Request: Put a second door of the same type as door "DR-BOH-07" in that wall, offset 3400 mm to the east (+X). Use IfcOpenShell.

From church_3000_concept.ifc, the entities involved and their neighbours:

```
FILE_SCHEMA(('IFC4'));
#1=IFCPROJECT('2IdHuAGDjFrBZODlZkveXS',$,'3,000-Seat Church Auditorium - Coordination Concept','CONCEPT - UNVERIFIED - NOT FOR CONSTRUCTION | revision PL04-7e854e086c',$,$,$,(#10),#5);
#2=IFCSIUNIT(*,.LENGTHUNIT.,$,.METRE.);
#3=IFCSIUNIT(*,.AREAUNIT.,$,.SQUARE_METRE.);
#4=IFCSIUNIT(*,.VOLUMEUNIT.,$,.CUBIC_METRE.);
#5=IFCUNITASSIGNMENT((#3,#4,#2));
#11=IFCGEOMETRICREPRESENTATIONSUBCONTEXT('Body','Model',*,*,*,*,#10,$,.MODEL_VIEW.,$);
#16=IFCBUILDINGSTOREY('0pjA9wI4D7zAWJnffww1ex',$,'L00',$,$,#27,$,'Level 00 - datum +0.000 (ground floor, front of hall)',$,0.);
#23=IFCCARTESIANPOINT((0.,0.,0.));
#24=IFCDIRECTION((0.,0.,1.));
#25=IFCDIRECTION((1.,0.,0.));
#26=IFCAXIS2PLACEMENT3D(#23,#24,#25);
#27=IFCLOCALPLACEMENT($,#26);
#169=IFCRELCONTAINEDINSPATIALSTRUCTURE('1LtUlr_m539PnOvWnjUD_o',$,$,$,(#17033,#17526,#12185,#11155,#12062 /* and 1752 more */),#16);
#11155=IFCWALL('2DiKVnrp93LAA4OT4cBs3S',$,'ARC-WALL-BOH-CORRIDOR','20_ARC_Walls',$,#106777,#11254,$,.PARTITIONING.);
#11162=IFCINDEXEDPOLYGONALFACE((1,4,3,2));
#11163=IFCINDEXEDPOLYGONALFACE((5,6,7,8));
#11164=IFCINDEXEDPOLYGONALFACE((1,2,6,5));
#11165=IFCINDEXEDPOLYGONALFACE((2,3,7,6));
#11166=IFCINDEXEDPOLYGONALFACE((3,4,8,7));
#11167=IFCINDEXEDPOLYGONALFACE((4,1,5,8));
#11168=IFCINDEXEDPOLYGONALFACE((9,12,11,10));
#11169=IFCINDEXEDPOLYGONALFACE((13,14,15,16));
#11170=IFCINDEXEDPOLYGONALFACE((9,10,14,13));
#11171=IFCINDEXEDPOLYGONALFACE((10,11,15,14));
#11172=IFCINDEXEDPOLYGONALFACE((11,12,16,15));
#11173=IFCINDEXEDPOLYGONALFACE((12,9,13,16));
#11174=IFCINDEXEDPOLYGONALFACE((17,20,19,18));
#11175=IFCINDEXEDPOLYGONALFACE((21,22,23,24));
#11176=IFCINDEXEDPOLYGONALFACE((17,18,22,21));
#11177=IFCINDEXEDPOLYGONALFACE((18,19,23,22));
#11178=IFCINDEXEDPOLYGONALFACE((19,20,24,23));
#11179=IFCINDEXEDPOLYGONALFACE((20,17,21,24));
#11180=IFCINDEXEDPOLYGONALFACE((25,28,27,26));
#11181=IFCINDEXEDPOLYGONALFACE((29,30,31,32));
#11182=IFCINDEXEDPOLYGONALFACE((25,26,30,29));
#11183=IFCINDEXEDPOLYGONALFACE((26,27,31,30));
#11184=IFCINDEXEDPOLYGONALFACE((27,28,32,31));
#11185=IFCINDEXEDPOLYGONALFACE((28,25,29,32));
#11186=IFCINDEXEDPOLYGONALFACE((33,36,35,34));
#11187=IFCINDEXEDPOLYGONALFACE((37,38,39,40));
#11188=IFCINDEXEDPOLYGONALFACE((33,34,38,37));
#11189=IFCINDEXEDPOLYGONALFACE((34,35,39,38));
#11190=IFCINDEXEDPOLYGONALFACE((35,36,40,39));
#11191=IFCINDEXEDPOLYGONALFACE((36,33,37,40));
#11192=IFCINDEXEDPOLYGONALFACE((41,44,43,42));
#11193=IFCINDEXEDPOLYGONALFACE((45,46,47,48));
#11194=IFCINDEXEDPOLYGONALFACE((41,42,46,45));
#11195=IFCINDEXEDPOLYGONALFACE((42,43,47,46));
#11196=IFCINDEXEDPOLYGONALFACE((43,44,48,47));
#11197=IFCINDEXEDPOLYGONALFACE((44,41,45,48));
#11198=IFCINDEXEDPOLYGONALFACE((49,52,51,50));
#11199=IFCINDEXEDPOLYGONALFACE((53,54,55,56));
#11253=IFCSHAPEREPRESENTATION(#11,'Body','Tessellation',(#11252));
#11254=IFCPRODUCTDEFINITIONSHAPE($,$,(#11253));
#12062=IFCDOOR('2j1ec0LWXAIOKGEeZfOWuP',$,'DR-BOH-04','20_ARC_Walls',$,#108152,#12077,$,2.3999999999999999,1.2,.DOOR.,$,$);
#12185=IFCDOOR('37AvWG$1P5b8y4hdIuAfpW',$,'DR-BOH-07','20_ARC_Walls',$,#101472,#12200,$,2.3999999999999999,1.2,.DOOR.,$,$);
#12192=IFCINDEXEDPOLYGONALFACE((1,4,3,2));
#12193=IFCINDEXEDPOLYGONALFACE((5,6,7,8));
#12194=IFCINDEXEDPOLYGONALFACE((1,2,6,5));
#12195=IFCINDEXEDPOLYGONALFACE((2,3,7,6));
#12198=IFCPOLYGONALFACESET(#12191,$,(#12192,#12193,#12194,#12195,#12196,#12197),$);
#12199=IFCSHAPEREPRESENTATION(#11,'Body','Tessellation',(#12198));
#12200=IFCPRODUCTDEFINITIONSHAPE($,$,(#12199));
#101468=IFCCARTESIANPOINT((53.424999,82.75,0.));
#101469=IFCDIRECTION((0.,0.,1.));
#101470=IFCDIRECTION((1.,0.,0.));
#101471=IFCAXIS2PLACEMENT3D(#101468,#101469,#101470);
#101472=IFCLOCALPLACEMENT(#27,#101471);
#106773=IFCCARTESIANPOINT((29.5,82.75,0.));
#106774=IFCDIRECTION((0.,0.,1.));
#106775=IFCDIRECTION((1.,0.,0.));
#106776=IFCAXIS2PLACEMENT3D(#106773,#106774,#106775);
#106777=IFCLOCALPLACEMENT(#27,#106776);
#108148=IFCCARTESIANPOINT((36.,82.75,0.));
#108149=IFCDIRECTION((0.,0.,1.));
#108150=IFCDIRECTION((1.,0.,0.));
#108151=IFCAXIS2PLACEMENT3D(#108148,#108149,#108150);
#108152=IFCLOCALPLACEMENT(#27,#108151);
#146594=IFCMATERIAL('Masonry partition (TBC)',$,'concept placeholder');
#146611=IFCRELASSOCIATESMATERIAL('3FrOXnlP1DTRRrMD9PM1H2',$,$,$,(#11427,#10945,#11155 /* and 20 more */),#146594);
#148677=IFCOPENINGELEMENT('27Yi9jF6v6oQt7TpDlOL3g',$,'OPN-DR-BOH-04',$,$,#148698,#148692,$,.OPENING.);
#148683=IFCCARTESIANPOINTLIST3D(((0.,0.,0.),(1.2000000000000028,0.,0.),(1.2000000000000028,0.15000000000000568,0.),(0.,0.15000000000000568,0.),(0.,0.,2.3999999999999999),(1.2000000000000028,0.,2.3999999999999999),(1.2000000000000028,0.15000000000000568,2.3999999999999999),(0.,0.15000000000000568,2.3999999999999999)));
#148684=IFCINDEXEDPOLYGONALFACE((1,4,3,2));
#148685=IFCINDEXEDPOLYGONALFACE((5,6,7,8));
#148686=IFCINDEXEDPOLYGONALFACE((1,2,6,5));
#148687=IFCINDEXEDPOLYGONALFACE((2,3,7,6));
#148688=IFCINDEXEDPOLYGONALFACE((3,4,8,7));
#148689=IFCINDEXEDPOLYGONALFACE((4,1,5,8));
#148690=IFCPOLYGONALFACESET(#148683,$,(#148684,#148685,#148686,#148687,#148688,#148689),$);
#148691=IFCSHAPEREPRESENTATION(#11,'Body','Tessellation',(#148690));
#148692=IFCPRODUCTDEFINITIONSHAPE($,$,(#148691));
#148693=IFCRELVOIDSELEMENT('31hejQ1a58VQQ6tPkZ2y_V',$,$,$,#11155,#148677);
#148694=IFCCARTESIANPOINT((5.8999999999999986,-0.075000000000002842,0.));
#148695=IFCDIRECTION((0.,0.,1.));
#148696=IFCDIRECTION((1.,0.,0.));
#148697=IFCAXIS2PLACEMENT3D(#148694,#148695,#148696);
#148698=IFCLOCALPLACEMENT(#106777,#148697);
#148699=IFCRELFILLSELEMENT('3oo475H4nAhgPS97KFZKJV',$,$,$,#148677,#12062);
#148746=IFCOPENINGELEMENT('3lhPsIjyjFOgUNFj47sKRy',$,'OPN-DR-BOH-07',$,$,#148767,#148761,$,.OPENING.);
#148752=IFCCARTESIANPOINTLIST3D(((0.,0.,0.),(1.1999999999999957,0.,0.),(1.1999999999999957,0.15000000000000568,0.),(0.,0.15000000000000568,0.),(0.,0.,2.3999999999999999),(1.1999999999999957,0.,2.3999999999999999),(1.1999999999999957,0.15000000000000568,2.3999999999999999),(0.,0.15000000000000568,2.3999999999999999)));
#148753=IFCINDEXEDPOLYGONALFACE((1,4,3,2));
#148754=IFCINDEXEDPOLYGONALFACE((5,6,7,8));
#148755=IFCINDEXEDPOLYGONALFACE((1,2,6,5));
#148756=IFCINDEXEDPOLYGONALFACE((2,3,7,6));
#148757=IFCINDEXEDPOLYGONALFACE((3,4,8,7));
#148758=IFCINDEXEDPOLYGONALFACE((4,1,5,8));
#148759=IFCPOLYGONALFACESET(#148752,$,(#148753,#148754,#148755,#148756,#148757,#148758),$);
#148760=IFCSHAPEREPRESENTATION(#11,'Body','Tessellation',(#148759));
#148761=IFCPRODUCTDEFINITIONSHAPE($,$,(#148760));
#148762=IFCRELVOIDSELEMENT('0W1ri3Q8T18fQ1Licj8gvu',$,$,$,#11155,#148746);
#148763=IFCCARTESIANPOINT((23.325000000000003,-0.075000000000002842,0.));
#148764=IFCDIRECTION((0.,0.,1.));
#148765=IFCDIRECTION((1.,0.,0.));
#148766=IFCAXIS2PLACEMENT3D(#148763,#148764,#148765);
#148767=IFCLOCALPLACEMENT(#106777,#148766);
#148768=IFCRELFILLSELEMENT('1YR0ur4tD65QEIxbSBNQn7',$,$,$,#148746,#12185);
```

```python
import ifcopenshell
import ifcopenshell.api.feature
import ifcopenshell.api.geometry
import ifcopenshell.api.root
import ifcopenshell.geom
import ifcopenshell.util.element
import ifcopenshell.util.placement
import ifcopenshell.util.shape
import ifcopenshell.util.unit

model = ifcopenshell.open("church_3000_concept.ifc")
unit_scale = ifcopenshell.util.unit.calculate_unit_scale(model)
settings = ifcopenshell.geom.settings()


def volume(element):
    """Net volume in cubic metres, openings subtracted."""
    shape = ifcopenshell.geom.create_shape(settings, element)
    return ifcopenshell.util.shape.get_volume(shape.geometry)


door = model.by_guid("37AvWG$1P5b8y4hdIuAfpW")
opening = door.FillsVoids[0].RelatingOpeningElement
wall = opening.VoidsElements[0].RelatingBuildingElement
before = volume(wall)
shift = ifcopenshell.util.placement.get_local_placement(wall.ObjectPlacement)[:3, 0] * 3.4 / unit_scale

# copy_class copies the void relationship, type, container and properties, but no geometry.
new_opening = ifcopenshell.api.root.copy_class(model, product=opening)
new_opening.Representation = ifcopenshell.util.element.copy_deep(
    model, opening.Representation, exclude=["IfcGeometricRepresentationContext", "IfcRepresentationMap"]
)
new_door = ifcopenshell.api.root.copy_class(model, product=door)
new_door.Representation = ifcopenshell.util.element.copy_deep(
    model, door.Representation, exclude=["IfcGeometricRepresentationContext", "IfcRepresentationMap"]
)
ifcopenshell.api.feature.add_filling(model, opening=new_opening, element=new_door)

for old, new in ((opening, new_opening), (door, new_door)):
    matrix = ifcopenshell.util.placement.get_local_placement(old.ObjectPlacement)
    matrix[:3, 3] += shift
    ifcopenshell.api.geometry.edit_object_placement(model, product=new, matrix=matrix, is_si=False)

after = volume(wall)

print(f"wall volume {before:.3f} -> {after:.3f} m3")

model.write("church_3000_concept_updated.ifc")
```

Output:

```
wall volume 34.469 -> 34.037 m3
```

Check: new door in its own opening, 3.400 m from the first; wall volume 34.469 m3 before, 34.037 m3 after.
